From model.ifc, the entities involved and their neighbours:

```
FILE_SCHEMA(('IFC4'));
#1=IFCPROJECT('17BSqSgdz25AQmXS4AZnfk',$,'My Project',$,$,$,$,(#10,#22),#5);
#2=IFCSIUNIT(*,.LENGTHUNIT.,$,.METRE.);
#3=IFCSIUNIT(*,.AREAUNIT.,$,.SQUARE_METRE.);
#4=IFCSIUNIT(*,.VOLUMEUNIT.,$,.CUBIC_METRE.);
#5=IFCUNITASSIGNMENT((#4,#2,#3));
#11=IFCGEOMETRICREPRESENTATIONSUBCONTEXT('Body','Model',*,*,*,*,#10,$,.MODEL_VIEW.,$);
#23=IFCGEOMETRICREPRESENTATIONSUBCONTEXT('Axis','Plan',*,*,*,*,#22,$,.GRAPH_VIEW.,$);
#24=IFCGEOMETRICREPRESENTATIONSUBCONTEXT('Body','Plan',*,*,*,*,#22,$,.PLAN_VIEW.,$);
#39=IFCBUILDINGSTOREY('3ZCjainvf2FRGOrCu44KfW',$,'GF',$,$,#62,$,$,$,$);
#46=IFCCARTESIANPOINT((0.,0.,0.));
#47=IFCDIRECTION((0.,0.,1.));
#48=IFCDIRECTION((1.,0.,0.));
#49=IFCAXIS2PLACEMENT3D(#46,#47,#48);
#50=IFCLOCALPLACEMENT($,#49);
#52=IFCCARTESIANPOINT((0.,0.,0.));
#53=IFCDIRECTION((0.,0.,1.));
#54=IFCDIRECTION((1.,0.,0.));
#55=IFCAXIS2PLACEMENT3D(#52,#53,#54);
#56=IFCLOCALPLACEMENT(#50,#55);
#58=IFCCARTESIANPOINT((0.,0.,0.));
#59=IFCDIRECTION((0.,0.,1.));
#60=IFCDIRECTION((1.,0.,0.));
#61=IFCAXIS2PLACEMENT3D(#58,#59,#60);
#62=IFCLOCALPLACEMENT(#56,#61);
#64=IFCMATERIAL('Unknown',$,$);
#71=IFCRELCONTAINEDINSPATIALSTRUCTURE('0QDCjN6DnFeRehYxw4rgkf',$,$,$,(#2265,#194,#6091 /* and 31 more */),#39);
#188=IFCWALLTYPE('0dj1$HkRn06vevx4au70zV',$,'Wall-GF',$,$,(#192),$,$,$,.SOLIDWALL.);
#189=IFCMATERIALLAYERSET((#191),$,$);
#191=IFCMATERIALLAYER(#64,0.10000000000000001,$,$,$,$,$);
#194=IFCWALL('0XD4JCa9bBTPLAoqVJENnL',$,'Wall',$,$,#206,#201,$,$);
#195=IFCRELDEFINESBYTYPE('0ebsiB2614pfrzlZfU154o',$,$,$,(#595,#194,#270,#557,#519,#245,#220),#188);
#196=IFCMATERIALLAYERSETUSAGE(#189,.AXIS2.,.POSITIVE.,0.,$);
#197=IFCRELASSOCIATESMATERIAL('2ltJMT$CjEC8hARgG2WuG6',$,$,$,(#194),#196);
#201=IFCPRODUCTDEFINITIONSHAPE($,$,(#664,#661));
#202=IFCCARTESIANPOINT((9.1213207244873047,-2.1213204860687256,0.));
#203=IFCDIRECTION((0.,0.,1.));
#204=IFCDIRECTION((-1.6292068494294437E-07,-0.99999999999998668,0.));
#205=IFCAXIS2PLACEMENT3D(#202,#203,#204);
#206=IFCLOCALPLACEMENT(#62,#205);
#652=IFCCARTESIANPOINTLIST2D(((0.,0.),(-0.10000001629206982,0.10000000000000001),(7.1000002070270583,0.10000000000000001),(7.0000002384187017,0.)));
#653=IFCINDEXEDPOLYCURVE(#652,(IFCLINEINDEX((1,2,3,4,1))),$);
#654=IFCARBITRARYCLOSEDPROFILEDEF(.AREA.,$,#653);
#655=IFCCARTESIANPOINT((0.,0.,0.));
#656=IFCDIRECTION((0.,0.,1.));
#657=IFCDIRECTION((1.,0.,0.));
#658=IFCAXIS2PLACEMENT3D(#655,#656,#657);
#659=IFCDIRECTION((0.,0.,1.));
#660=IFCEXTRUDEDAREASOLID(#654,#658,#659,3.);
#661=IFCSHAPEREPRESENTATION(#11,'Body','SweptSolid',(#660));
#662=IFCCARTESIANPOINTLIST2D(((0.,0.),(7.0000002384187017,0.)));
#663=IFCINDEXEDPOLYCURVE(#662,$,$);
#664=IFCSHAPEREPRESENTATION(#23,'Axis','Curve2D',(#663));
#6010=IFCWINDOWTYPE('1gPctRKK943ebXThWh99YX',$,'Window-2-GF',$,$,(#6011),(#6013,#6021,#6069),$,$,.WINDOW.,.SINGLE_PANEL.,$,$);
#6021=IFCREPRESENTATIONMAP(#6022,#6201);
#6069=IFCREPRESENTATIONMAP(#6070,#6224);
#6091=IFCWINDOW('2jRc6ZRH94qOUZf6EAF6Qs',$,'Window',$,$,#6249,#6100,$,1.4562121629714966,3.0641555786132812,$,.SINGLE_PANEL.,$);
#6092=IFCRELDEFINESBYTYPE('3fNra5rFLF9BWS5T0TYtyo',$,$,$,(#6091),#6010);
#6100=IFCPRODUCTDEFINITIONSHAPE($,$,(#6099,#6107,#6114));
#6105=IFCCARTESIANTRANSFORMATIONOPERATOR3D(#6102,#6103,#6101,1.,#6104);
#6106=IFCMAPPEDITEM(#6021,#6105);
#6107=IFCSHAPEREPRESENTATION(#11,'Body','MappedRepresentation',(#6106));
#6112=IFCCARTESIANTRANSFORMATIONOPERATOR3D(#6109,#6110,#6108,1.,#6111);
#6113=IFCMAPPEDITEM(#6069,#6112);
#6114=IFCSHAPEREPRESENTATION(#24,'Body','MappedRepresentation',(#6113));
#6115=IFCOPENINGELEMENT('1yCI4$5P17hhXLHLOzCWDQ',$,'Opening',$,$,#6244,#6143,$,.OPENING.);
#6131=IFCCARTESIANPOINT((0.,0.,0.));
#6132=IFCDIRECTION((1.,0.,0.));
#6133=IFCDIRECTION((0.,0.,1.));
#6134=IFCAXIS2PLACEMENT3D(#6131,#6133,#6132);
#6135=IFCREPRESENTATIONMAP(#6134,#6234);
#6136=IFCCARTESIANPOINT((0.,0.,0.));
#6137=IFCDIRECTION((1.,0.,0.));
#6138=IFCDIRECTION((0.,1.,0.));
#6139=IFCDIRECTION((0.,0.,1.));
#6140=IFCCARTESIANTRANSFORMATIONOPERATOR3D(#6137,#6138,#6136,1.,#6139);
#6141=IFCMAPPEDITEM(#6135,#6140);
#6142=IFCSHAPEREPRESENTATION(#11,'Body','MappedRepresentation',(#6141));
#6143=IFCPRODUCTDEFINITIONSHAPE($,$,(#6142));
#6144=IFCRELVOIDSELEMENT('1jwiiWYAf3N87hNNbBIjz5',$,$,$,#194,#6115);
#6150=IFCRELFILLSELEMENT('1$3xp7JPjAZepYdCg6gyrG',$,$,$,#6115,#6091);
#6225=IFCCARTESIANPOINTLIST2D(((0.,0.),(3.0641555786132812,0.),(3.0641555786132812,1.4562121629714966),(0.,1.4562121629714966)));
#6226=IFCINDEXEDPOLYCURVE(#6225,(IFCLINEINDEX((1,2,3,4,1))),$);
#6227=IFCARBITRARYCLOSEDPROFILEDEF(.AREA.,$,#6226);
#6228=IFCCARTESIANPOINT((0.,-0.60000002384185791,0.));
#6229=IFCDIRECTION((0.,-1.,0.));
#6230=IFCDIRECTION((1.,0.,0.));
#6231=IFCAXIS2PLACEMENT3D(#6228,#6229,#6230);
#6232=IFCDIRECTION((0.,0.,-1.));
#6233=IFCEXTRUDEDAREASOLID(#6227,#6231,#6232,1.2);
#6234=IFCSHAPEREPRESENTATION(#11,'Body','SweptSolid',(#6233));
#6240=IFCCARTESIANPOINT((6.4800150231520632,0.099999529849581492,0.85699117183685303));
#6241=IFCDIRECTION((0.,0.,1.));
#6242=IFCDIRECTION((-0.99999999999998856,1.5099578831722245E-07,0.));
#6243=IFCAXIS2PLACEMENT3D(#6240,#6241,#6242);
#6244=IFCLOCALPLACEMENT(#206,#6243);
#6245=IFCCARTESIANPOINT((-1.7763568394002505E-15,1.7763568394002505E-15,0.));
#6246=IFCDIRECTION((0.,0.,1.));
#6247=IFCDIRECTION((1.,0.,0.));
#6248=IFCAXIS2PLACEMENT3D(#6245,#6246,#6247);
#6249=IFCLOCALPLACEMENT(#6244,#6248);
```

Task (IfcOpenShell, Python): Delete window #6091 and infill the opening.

```python
import ifcopenshell
import ifcopenshell.api.feature
import ifcopenshell.api.root
import ifcopenshell.geom
import ifcopenshell.util.shape

model = ifcopenshell.open("model.ifc")
settings = ifcopenshell.geom.settings()


def volume(element):
    """Net volume in cubic metres, openings subtracted."""
    shape = ifcopenshell.geom.create_shape(settings, element)
    return ifcopenshell.util.shape.get_volume(shape.geometry)


window = model.by_guid("2jRc6ZRH94qOUZf6EAF6Qs")
opening = window.FillsVoids[0].RelatingOpeningElement
wall = opening.VoidsElements[0].RelatingBuildingElement
before = volume(wall)

ifcopenshell.api.root.remove_product(model, product=window)
ifcopenshell.api.feature.remove_feature(model, feature=opening)

after = volume(wall)

print(f"wall volume {before:.3f} -> {after:.3f} m3")

model.write("model_v2.ifc")
```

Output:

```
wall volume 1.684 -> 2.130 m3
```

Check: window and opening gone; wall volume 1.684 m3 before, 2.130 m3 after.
